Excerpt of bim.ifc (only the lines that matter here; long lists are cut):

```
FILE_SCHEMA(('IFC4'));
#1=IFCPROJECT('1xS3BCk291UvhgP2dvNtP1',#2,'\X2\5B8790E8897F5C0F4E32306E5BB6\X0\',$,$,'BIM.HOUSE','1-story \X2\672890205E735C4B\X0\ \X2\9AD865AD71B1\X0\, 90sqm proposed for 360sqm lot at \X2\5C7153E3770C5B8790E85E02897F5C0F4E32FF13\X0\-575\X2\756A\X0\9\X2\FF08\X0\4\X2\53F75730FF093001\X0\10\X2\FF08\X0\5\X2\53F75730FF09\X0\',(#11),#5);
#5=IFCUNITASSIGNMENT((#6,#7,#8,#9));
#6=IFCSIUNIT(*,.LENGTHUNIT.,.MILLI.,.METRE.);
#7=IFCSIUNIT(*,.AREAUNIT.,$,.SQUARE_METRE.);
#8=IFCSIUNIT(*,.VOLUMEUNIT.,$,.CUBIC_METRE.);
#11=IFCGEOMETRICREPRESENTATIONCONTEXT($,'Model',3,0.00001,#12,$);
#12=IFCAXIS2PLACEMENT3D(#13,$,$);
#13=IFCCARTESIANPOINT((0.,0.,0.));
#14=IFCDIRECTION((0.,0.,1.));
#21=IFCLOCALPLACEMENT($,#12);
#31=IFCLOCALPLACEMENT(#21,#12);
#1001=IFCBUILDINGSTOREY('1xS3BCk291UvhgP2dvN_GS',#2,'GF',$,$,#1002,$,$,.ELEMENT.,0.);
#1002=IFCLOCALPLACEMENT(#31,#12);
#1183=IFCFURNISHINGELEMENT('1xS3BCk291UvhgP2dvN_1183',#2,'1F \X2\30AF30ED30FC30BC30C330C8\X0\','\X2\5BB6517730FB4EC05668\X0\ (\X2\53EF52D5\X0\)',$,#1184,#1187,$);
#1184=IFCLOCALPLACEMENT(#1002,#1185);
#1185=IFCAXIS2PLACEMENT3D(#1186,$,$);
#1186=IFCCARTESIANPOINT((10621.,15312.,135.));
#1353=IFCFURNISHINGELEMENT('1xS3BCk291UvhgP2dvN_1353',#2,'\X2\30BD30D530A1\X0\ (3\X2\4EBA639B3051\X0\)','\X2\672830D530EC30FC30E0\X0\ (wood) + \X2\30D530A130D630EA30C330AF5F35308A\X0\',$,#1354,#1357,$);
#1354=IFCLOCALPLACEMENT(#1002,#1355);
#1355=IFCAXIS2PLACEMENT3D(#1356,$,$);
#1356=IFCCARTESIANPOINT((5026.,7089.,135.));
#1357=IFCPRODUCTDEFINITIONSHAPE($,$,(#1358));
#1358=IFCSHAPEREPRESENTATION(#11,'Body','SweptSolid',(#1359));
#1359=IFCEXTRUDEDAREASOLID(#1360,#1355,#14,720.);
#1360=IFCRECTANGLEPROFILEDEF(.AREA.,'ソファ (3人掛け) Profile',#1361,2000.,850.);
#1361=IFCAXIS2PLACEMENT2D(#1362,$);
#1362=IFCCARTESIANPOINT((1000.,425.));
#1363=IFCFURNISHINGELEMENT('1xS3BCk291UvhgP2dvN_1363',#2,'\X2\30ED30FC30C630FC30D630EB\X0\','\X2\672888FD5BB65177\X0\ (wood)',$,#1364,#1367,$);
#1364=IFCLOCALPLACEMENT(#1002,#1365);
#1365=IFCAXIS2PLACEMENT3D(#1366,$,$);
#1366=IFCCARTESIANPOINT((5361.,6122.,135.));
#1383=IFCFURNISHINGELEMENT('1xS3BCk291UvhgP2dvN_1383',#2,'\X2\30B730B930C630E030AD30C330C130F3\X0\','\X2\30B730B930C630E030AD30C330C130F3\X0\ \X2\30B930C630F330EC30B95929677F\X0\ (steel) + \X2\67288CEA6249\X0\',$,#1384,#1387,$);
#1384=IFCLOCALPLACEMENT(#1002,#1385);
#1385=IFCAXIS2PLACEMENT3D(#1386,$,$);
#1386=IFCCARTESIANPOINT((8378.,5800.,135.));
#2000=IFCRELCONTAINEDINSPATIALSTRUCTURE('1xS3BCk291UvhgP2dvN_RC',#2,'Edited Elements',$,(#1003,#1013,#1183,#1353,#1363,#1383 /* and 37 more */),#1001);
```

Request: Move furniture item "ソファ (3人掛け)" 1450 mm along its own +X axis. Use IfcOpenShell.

```python
import ifcopenshell
import ifcopenshell.api.geometry
import ifcopenshell.util.placement
import ifcopenshell.util.unit

model = ifcopenshell.open("bim.ifc")
unit_scale = ifcopenshell.util.unit.calculate_unit_scale(model)

item = model.by_guid("1xS3BCk291UvhgP2dvN_1353")
matrix = ifcopenshell.util.placement.get_local_placement(item.ObjectPlacement)
matrix[:3, 3] += matrix[:3, 0] * 1.45 / unit_scale
ifcopenshell.api.geometry.edit_object_placement(model, product=item, matrix=matrix, is_si=False)

print(ifcopenshell.util.placement.get_local_placement(item.ObjectPlacement).round(3) + 0.0)

model.write("bim_v2.ifc")
```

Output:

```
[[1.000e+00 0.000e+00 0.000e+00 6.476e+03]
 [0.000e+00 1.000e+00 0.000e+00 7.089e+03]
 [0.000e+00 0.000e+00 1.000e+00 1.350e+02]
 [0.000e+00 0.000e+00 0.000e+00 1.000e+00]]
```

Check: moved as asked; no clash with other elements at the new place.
